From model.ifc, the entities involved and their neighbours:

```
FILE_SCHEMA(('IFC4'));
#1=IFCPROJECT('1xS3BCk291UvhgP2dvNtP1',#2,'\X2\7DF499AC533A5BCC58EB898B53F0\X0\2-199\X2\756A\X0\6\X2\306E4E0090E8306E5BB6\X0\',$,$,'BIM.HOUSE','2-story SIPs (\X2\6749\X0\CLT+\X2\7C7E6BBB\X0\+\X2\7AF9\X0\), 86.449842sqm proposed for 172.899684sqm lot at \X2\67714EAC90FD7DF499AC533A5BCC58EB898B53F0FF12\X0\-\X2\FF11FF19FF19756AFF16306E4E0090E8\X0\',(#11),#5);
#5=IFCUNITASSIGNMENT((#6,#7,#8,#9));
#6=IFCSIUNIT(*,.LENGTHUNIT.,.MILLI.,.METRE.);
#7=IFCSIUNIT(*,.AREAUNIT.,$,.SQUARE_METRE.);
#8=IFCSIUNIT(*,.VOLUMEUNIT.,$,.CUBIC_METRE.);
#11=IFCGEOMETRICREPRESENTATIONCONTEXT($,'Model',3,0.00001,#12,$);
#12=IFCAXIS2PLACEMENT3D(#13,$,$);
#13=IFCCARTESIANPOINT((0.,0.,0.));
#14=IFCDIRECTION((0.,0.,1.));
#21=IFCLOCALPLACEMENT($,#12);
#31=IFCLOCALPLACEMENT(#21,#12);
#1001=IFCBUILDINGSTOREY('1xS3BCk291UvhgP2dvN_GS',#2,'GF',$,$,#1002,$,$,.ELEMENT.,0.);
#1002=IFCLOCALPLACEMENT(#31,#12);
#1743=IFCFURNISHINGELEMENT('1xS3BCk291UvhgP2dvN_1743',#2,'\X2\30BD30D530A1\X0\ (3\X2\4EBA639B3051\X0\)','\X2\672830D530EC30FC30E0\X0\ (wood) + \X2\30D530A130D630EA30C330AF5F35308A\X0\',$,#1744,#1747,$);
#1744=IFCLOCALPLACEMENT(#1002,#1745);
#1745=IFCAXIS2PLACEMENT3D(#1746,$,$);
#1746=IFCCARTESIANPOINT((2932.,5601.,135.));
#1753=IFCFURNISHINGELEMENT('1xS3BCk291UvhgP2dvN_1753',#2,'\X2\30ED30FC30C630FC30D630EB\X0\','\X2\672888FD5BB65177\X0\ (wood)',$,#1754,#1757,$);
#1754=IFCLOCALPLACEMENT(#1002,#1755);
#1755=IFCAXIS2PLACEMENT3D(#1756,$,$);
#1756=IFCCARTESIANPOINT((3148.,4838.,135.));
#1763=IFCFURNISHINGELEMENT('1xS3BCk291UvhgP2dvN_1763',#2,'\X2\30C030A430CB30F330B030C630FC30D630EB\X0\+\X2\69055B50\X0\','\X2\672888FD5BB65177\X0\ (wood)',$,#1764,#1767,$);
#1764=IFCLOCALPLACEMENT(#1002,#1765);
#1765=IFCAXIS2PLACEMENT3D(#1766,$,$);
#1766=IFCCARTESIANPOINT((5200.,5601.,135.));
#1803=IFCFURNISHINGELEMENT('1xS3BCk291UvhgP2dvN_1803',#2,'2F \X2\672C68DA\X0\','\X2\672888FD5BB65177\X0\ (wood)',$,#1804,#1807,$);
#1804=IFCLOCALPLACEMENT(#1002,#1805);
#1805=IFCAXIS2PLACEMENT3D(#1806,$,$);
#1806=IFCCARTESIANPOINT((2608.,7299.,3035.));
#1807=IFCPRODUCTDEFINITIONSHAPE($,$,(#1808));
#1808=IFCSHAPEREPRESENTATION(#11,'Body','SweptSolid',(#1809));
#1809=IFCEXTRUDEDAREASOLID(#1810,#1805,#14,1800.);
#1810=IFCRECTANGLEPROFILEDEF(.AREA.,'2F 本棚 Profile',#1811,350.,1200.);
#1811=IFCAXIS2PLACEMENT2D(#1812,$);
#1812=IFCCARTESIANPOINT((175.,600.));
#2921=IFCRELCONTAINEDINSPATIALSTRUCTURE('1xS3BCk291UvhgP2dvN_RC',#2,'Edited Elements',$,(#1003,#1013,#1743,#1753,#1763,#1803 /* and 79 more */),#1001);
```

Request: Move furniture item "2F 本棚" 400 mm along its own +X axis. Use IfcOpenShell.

```python
import ifcopenshell
import ifcopenshell.api.geometry
import ifcopenshell.util.placement

model = ifcopenshell.open("model.ifc")

item = model.by_guid("1xS3BCk291UvhgP2dvN_1803")
matrix = ifcopenshell.util.placement.get_local_placement(item.ObjectPlacement)
matrix[:3, 3] += matrix[:3, 0] * 400.0
ifcopenshell.api.geometry.edit_object_placement(model, product=item, matrix=matrix, is_si=False)

print(ifcopenshell.util.placement.get_local_placement(item.ObjectPlacement).round(3) + 0.0)

model.write("model_rev.ifc")
```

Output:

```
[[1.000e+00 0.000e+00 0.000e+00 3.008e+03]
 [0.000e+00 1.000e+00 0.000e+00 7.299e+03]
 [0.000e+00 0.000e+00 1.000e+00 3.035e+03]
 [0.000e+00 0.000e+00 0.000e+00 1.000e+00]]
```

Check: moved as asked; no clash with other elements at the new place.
